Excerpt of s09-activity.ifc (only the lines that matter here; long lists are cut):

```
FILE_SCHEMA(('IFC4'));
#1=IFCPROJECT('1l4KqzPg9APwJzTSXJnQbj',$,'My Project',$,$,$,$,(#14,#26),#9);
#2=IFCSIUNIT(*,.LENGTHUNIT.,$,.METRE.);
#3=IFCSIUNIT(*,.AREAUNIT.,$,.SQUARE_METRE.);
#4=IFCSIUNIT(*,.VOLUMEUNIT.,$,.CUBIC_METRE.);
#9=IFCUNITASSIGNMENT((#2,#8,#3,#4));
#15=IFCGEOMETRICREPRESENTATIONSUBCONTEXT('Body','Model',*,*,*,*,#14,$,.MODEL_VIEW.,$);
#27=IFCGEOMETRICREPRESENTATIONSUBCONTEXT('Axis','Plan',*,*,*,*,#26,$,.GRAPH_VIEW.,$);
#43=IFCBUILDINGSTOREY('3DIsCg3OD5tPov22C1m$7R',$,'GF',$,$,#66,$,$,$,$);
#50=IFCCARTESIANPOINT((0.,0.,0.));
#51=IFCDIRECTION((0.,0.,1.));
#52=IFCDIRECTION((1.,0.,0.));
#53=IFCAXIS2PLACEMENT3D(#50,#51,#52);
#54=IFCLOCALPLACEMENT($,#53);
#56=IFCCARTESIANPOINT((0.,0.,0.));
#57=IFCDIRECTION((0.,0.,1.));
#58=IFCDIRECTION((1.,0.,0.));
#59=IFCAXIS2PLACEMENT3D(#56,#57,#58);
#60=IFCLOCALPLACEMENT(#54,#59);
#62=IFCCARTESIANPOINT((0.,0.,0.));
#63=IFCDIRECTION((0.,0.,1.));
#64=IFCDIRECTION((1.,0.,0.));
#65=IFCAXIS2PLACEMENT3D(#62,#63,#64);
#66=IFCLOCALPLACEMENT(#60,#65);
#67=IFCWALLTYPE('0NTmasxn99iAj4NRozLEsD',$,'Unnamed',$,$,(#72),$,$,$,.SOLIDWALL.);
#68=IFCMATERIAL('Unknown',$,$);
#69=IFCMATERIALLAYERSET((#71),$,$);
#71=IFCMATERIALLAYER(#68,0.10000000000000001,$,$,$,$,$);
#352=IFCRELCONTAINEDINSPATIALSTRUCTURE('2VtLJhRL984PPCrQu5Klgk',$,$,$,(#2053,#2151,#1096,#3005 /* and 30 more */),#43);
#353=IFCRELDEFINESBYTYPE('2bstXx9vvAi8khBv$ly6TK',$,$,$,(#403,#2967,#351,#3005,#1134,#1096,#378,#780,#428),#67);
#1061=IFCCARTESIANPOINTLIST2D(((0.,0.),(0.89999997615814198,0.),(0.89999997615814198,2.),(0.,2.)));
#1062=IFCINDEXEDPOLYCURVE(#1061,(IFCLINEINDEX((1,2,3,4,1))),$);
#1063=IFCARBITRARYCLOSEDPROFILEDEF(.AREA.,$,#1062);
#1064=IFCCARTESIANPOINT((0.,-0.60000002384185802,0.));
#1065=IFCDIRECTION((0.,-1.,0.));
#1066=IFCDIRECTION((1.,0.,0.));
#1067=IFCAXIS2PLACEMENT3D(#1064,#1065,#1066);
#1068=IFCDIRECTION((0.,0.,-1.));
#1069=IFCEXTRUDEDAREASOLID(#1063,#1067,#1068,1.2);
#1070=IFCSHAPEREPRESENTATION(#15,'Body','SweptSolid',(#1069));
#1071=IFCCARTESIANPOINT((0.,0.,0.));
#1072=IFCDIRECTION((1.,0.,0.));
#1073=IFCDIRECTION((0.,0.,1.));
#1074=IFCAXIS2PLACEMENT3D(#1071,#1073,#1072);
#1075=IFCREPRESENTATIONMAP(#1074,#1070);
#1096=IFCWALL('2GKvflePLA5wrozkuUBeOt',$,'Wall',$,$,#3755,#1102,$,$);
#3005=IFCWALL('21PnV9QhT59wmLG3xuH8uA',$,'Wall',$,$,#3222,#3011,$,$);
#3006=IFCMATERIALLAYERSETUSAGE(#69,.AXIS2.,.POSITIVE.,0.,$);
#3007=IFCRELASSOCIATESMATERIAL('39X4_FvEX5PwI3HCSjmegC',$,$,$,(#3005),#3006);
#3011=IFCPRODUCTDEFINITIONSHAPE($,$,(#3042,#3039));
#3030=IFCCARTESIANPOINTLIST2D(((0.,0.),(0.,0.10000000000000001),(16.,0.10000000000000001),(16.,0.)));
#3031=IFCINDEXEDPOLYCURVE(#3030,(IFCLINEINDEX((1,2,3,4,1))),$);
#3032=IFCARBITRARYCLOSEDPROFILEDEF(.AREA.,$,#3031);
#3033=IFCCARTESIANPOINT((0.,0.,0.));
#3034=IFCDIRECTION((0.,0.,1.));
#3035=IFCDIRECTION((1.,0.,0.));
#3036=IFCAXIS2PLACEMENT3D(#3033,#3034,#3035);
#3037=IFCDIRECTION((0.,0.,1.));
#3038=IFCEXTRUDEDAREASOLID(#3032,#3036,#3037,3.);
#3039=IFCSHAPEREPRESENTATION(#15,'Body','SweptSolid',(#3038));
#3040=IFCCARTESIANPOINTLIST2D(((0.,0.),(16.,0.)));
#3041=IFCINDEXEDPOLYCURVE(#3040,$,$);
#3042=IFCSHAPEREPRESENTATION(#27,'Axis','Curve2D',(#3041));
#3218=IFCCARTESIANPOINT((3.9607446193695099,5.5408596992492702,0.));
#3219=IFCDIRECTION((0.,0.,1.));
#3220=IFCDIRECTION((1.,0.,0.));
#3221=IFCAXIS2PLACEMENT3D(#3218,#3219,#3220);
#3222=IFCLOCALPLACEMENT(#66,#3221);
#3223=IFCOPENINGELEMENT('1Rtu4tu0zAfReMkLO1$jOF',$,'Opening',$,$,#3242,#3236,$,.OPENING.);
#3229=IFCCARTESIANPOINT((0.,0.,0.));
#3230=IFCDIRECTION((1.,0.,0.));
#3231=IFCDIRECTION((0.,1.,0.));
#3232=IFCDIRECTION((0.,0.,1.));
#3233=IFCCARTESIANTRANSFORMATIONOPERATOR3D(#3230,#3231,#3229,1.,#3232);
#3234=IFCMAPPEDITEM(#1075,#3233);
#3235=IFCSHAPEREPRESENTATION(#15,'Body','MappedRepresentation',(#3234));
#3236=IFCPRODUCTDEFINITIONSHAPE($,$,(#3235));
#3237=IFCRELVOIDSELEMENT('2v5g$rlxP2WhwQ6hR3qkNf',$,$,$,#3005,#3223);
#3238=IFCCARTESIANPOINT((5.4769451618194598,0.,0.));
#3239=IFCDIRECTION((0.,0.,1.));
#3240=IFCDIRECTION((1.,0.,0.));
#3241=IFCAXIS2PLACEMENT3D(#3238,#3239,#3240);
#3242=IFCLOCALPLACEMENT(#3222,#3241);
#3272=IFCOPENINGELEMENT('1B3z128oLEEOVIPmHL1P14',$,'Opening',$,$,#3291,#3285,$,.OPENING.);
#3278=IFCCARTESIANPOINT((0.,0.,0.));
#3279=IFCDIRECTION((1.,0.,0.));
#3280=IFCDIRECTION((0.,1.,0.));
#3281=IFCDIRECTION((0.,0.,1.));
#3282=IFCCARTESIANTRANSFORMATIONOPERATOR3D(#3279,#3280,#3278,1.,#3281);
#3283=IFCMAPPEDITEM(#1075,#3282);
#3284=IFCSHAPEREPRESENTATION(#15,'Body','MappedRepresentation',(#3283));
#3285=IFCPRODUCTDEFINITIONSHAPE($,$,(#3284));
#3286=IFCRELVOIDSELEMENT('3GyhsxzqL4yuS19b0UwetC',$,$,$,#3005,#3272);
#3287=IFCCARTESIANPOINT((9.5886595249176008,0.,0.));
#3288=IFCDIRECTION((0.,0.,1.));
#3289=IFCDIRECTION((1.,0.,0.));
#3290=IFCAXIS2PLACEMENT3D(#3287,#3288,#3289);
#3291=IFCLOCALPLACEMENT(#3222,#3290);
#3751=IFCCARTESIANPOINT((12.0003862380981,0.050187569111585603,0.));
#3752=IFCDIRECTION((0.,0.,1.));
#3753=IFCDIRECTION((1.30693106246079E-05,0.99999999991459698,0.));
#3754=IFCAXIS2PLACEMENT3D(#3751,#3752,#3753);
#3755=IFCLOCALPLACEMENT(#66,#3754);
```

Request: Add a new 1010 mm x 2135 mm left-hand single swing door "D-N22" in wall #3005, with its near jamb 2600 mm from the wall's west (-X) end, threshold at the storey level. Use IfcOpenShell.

```python
import numpy as np
import ifcopenshell
import ifcopenshell.api.feature
import ifcopenshell.api.geometry
import ifcopenshell.api.root
import ifcopenshell.api.spatial
import ifcopenshell.geom
import ifcopenshell.util.element
import ifcopenshell.util.placement
import ifcopenshell.util.representation
import ifcopenshell.util.shape
import ifcopenshell.util.unit

model = ifcopenshell.open("s09-activity.ifc")
unit_scale = ifcopenshell.util.unit.calculate_unit_scale(model)
settings = ifcopenshell.geom.settings()


def volume(element):
    """Net volume in cubic metres, openings subtracted."""
    shape = ifcopenshell.geom.create_shape(settings, element)
    return ifcopenshell.util.shape.get_volume(shape.geometry)


wall = model.by_guid("21PnV9QhT59wmLG3xuH8uA")
storey = ifcopenshell.util.element.get_container(wall, ifc_class="IfcBuildingStorey")
context = ifcopenshell.util.representation.get_context(model, "Model", "Body", "MODEL_VIEW")
before = volume(wall)

width, height, from_end, sill = 1.01, 2.135, 2.6, 0.0  # metres

# The wall runs along its own X axis, and the end named is its -X end.
wall_shape = ifcopenshell.geom.create_shape(settings, wall)
x, y, z = ifcopenshell.util.shape.get_vertices(wall_shape.geometry).T
start = x.min() + from_end
face, thickness = float(y.min()), float(y.max() - y.min())
wall_matrix = ifcopenshell.util.placement.get_local_placement(wall.ObjectPlacement)
level = ifcopenshell.util.placement.get_local_placement(storey.ObjectPlacement)[2, 3]


def in_wall(x, y):
    """Placement at x, y metres in the wall's axes, at sill height."""
    matrix = wall_matrix.copy()
    matrix[:, 3] = wall_matrix @ np.array([x / unit_scale, y / unit_scale, 0.0, 1.0])
    matrix[2, 3] = level + sill / unit_scale
    return matrix


# Opening: a box that overshoots both wall faces by 50 mm.
opening = ifcopenshell.api.root.create_entity(model, ifc_class="IfcOpeningElement", predefined_type="OPENING")
box = ifcopenshell.api.geometry.add_wall_representation(
    model, context=context, length=width, height=height, thickness=thickness + 0.1
)
ifcopenshell.api.geometry.assign_representation(model, product=opening, representation=box)
ifcopenshell.api.geometry.edit_object_placement(model, product=opening, matrix=in_wall(start, face - 0.05), is_si=False)
ifcopenshell.api.feature.add_feature(model, feature=opening, element=wall)

door = ifcopenshell.api.root.create_entity(model, ifc_class="IfcDoor", name="D-N22", predefined_type="DOOR")
door.OverallWidth, door.OverallHeight = width / unit_scale, height / unit_scale
door.OperationType = "SINGLE_SWING_LEFT"
body = ifcopenshell.api.geometry.add_door_representation(
    model,
    context=context,
    overall_width=door.OverallWidth,
    overall_height=door.OverallHeight,
    operation_type="SINGLE_SWING_LEFT",
    lining_properties={"LiningDepth": thickness / unit_scale, "ThresholdDepth": thickness / unit_scale},
)
ifcopenshell.api.geometry.assign_representation(model, product=door, representation=body)
ifcopenshell.api.spatial.assign_container(model, products=[door], relating_structure=storey)
ifcopenshell.api.feature.add_filling(model, opening=opening, element=door)

# The lining spans the wall, so the door starts at the wall face.
ifcopenshell.api.geometry.edit_object_placement(model, product=door, matrix=in_wall(start, face), is_si=False)

after = volume(wall)

print(f"wall volume {before:.3f} -> {after:.3f} m3")

model.write("s09-activity_edited.ifc")
```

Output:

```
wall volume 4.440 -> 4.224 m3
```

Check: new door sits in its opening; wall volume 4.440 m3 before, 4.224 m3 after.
